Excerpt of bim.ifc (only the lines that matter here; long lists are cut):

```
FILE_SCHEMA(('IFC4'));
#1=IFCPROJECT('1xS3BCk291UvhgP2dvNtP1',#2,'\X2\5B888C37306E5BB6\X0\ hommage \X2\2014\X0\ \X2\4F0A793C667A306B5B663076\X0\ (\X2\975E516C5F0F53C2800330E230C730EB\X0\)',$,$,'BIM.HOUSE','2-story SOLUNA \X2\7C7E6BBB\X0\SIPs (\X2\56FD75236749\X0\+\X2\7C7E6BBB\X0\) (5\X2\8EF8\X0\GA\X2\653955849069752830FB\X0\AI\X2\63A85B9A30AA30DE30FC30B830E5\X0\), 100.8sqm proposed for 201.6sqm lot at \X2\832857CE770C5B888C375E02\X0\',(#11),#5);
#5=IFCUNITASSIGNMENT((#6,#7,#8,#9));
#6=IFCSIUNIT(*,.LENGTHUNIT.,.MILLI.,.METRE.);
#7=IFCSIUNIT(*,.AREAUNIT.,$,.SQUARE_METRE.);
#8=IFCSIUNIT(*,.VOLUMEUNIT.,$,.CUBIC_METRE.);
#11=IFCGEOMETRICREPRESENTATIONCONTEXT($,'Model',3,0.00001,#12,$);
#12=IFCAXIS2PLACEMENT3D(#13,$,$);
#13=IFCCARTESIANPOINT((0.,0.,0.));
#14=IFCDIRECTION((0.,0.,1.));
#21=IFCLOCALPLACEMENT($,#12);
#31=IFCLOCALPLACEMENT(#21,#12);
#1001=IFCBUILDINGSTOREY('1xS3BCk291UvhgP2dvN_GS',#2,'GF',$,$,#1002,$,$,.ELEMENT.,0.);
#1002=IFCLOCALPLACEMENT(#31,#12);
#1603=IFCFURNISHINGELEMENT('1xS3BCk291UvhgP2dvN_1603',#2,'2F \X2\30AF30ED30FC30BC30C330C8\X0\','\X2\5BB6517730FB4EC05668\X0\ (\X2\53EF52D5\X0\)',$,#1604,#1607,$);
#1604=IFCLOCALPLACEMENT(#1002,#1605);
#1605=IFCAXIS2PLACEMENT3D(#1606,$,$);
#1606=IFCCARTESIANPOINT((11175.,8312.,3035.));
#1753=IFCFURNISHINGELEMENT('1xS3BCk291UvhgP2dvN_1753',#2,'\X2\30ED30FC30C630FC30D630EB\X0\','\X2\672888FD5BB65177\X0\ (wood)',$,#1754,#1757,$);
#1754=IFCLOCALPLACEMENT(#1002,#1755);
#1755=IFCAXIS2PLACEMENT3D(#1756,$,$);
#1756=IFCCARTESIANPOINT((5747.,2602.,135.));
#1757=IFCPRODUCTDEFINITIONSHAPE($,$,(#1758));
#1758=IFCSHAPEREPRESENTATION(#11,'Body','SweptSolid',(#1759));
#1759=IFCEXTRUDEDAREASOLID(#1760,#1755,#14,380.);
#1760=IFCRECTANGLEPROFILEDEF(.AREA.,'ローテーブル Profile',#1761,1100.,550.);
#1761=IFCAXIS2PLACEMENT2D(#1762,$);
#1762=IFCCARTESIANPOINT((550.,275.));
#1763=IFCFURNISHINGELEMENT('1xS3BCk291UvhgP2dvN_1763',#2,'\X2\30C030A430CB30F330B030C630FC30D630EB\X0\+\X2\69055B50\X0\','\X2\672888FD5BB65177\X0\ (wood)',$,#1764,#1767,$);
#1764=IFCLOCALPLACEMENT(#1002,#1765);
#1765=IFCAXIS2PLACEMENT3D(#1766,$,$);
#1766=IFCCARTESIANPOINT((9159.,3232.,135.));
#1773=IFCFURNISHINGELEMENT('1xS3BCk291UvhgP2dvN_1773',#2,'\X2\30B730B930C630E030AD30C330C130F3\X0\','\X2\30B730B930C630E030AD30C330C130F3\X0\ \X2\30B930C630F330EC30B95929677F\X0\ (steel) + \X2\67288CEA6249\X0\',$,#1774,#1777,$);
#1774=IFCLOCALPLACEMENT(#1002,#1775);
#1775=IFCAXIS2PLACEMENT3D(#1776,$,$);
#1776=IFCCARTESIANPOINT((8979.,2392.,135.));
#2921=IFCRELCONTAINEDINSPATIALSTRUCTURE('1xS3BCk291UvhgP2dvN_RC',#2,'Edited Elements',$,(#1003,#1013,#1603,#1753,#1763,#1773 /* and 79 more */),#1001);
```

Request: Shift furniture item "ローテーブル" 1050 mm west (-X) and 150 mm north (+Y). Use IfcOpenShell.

```python
import ifcopenshell
import ifcopenshell.api.geometry
import ifcopenshell.util.placement

model = ifcopenshell.open("bim.ifc")

item = model.by_id(1753)
matrix = ifcopenshell.util.placement.get_local_placement(item.ObjectPlacement)
matrix[0, 3] -= 1050.0
matrix[1, 3] += 150.0
ifcopenshell.api.geometry.edit_object_placement(model, product=item, matrix=matrix, is_si=False)

print(ifcopenshell.util.placement.get_local_placement(item.ObjectPlacement).round(3) + 0.0)

model.write("bim_v2.ifc")
```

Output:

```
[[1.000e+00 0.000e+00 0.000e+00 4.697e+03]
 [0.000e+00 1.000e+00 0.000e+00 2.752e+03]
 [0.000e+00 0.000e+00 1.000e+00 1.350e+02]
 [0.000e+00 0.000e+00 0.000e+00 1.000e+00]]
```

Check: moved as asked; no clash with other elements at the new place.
